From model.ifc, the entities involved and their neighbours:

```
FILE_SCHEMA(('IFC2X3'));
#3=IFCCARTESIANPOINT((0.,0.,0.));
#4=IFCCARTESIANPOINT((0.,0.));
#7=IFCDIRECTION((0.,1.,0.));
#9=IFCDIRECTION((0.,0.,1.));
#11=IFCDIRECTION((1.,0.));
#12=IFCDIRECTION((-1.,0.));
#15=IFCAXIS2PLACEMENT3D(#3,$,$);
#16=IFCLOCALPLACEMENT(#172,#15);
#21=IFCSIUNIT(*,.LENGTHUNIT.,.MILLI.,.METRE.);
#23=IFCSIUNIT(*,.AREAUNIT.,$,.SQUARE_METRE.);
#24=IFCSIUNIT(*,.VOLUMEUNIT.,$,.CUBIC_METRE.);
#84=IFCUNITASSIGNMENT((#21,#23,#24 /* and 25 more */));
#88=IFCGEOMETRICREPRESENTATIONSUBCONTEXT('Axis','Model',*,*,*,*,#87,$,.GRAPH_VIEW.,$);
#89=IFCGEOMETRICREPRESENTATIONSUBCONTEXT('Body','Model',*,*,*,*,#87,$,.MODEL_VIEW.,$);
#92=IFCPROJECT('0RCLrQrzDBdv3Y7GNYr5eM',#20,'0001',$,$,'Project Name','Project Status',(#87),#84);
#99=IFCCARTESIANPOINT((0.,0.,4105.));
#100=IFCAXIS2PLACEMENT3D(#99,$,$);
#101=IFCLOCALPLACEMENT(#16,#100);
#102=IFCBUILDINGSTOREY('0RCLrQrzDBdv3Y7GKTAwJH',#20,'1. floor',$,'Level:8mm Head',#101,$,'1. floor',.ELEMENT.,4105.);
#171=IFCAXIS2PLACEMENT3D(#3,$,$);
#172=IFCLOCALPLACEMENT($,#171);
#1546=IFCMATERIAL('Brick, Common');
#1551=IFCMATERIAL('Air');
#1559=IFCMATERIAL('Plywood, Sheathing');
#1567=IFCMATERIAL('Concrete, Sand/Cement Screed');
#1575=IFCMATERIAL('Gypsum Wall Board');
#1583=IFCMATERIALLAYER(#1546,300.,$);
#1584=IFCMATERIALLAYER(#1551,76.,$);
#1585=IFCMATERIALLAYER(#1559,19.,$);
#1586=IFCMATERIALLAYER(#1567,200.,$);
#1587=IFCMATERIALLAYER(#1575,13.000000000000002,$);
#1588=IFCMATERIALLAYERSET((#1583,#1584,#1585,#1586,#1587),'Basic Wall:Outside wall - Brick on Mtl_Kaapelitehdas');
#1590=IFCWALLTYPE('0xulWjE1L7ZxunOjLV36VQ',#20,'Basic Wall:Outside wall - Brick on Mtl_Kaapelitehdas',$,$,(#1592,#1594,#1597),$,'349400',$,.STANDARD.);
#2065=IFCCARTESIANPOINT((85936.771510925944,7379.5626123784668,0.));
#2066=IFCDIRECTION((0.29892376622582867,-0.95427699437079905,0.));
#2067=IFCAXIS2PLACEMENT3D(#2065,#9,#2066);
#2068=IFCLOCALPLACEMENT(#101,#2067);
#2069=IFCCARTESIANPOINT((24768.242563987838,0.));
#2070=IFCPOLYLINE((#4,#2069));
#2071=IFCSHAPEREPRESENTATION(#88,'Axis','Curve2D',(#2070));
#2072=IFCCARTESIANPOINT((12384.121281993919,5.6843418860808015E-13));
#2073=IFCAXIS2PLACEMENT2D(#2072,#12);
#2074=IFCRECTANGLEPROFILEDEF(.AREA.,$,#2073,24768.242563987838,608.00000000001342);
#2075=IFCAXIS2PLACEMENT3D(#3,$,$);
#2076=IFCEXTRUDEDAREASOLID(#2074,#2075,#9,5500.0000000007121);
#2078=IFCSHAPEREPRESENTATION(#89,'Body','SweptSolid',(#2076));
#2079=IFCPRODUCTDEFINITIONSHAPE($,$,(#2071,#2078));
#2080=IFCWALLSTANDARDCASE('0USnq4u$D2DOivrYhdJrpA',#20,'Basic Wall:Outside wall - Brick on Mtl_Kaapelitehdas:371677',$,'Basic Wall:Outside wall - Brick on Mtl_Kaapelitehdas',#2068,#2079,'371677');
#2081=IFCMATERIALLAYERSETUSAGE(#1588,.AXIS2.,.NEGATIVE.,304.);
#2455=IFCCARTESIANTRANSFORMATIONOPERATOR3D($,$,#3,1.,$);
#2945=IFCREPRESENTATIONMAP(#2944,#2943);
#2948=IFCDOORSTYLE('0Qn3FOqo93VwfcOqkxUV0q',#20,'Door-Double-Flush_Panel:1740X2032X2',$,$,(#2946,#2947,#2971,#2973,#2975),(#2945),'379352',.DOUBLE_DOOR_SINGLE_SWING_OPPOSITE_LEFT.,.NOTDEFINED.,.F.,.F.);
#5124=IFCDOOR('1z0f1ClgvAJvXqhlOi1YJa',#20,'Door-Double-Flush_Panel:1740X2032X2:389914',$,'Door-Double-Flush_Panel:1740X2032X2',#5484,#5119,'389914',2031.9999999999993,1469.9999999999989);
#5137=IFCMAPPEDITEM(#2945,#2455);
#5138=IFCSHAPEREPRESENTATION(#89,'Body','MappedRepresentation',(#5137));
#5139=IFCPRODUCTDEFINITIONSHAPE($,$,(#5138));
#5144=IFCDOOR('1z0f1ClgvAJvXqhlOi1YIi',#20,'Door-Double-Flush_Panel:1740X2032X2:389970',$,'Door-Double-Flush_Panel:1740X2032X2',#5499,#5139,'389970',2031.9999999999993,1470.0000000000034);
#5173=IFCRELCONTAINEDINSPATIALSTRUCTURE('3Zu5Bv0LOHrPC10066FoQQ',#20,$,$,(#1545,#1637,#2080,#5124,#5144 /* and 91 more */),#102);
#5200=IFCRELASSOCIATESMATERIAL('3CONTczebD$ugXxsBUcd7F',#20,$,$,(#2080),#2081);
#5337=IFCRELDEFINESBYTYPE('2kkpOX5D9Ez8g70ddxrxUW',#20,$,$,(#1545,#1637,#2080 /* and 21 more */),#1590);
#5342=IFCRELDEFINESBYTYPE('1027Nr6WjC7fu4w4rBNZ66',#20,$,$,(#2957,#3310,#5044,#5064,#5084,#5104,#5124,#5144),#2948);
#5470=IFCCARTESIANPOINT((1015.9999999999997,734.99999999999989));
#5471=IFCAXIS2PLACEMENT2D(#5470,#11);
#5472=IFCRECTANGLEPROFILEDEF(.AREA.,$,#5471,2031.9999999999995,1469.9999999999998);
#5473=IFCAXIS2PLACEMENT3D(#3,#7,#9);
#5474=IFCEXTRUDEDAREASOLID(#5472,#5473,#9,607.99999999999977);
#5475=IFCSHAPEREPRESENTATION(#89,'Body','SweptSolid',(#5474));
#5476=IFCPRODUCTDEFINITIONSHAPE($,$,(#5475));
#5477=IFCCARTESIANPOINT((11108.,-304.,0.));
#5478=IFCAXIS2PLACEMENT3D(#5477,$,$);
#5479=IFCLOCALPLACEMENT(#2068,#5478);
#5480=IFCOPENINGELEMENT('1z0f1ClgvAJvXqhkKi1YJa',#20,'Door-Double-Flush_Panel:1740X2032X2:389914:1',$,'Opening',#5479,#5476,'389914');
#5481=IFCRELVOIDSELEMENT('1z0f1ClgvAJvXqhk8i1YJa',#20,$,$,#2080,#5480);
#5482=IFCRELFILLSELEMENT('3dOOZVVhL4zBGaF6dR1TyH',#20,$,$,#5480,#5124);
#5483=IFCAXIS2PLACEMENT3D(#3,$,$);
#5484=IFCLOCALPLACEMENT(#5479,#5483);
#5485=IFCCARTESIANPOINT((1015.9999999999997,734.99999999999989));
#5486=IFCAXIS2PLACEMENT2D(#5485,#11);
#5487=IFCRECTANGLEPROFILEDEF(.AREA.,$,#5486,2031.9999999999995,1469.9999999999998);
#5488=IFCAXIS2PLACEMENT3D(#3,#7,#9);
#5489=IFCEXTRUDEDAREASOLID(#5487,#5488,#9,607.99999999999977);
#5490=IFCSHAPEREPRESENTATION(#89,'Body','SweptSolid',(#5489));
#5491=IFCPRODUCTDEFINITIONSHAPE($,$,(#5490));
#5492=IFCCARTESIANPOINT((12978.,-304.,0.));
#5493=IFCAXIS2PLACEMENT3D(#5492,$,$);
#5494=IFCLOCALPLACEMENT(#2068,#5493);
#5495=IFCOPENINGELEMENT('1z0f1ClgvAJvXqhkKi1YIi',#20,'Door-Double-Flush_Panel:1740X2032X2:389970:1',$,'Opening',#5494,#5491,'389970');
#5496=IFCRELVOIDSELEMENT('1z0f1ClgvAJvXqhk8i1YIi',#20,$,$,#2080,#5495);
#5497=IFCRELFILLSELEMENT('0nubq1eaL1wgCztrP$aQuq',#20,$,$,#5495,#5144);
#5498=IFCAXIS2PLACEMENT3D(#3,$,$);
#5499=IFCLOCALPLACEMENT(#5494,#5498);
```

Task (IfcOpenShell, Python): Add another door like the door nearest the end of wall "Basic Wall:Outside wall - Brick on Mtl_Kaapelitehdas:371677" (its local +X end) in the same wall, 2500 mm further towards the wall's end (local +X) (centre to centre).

```python
import ifcopenshell
import ifcopenshell.api.feature
import ifcopenshell.api.geometry
import ifcopenshell.api.root
import ifcopenshell.geom
import ifcopenshell.util.element
import ifcopenshell.util.placement
import ifcopenshell.util.shape
import ifcopenshell.util.unit

model = ifcopenshell.open("model.ifc")
unit_scale = ifcopenshell.util.unit.calculate_unit_scale(model)
settings = ifcopenshell.geom.settings()


def volume(element):
    """Net volume in cubic metres, openings subtracted."""
    shape = ifcopenshell.geom.create_shape(settings, element)
    return ifcopenshell.util.shape.get_volume(shape.geometry)


def reuse_history(source, copy):
    """copy_class also copies each property set's owner history, people and application; keep the originals."""
    for rel in copy.IsDefinedBy:
        if rel.is_a("IfcRelDefinesByProperties") and (history := rel.RelatingPropertyDefinition.OwnerHistory):
            rel.RelatingPropertyDefinition.OwnerHistory = source.OwnerHistory
            ifcopenshell.util.element.remove_deep2(model, history)


door = model.by_guid("1z0f1ClgvAJvXqhlOi1YIi")
opening = door.FillsVoids[0].RelatingOpeningElement
wall = opening.VoidsElements[0].RelatingBuildingElement
before = volume(wall)
shift = ifcopenshell.util.placement.get_local_placement(wall.ObjectPlacement)[:3, 0] * 2.5 / unit_scale

# copy_class copies the void relationship, type, container and properties, but no geometry.
new_opening = ifcopenshell.api.root.copy_class(model, product=opening)
new_opening.Representation = ifcopenshell.util.element.copy_deep(
    model, opening.Representation, exclude=["IfcGeometricRepresentationContext", "IfcRepresentationMap"]
)
new_opening.Name = "Door-Double-Flush_Panel:1740X2032X2"
new_opening.Tag = None
new_door = ifcopenshell.api.root.copy_class(model, product=door)
new_door.Representation = ifcopenshell.util.element.copy_deep(
    model, door.Representation, exclude=["IfcGeometricRepresentationContext", "IfcRepresentationMap"]
)
new_door.Name = "Door-Double-Flush_Panel:1740X2032X2"
new_door.Tag = None
reuse_history(door, new_door)
fills = ifcopenshell.api.feature.add_filling(model, opening=new_opening, element=new_door)
fills.OwnerHistory = new_door.OwnerHistory  # required in IFC2X3

for old, new in ((opening, new_opening), (door, new_door)):
    matrix = ifcopenshell.util.placement.get_local_placement(old.ObjectPlacement)
    matrix[:3, 3] += shift
    ifcopenshell.api.geometry.edit_object_placement(model, product=new, matrix=matrix, is_si=False)

after = volume(wall)

print(f"wall volume {before:.3f} -> {after:.3f} m3")

model.write("model_edited.ifc")
```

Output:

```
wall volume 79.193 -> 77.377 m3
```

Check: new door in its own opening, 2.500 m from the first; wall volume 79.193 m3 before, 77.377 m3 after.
